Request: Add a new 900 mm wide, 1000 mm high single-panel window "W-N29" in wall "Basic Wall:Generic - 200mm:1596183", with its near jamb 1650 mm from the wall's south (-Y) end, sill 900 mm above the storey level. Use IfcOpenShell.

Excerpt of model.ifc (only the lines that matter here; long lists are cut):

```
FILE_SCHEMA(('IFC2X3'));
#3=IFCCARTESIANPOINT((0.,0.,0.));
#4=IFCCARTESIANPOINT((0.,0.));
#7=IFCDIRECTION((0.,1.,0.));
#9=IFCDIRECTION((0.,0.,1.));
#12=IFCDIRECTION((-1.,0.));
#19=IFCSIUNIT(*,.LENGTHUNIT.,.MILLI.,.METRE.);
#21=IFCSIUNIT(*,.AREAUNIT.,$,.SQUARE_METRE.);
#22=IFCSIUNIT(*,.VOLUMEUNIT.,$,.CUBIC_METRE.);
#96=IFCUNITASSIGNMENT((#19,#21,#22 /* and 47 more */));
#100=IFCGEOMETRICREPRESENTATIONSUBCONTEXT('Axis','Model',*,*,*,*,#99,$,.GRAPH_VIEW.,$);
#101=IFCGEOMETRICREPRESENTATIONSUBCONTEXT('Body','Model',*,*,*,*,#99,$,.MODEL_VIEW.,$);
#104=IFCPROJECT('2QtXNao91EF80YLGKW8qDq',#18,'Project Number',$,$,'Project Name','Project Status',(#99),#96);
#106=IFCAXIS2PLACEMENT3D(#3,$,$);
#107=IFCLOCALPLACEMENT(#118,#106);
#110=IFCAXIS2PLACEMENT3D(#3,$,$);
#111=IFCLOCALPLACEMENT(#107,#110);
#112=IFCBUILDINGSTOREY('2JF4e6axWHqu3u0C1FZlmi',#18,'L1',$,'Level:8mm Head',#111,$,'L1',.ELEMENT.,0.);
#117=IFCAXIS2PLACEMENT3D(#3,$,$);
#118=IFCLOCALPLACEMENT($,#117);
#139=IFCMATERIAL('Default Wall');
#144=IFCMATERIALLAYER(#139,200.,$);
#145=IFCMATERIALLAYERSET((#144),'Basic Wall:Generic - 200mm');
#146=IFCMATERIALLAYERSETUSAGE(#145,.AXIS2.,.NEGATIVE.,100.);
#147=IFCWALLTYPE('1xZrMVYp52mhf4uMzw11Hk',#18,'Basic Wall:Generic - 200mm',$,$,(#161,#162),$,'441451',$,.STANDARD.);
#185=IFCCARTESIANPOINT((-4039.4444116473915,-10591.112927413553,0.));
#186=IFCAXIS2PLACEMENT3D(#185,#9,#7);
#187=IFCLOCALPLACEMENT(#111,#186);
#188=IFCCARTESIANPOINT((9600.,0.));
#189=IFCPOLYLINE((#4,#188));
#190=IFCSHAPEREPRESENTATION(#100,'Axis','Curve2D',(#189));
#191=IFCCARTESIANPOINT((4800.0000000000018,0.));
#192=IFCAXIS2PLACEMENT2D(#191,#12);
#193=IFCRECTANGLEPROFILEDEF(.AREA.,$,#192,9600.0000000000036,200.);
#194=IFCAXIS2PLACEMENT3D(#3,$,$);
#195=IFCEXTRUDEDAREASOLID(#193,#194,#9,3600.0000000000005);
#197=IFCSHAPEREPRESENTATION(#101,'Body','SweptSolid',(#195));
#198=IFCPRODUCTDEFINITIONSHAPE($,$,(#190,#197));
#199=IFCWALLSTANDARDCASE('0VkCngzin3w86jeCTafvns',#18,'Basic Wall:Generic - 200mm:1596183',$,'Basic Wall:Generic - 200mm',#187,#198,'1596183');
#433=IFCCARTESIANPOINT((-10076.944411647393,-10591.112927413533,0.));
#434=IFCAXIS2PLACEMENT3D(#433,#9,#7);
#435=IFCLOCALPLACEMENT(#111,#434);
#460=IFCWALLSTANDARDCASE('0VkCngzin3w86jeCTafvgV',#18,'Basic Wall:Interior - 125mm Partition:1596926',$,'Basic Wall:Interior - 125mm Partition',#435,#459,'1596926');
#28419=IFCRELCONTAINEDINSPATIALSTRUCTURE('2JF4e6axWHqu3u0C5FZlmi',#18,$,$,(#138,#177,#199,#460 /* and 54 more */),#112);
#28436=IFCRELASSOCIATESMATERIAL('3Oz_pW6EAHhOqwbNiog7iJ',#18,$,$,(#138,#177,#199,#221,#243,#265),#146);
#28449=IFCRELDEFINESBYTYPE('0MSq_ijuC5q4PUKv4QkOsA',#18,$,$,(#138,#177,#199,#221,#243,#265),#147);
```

```python
import numpy as np
import ifcopenshell
import ifcopenshell.api.feature
import ifcopenshell.api.geometry
import ifcopenshell.api.root
import ifcopenshell.api.spatial
import ifcopenshell.api.type
import ifcopenshell.geom
import ifcopenshell.util.element
import ifcopenshell.util.placement
import ifcopenshell.util.representation
import ifcopenshell.util.shape
import ifcopenshell.util.unit

model = ifcopenshell.open("model.ifc")
unit_scale = ifcopenshell.util.unit.calculate_unit_scale(model)
settings = ifcopenshell.geom.settings()


def volume(element):
    """Net volume in cubic metres, openings subtracted."""
    shape = ifcopenshell.geom.create_shape(settings, element)
    return ifcopenshell.util.shape.get_volume(shape.geometry)


wall = model.by_guid("0VkCngzin3w86jeCTafvns")
storey = ifcopenshell.util.element.get_container(wall, ifc_class="IfcBuildingStorey")
context = ifcopenshell.util.representation.get_context(model, "Model", "Body", "MODEL_VIEW")
before = volume(wall)

width, height, from_end, sill = 0.9, 1, 1.65, 0.9  # metres

# The wall runs along its own X axis, and the end named is its -X end.
wall_shape = ifcopenshell.geom.create_shape(settings, wall)
x, y, z = ifcopenshell.util.shape.get_vertices(wall_shape.geometry).T
start = x.min() + from_end
face, thickness = float(y.min()), float(y.max() - y.min())
wall_matrix = ifcopenshell.util.placement.get_local_placement(wall.ObjectPlacement)
level = ifcopenshell.util.placement.get_local_placement(storey.ObjectPlacement)[2, 3]


def in_wall(x, y):
    """Placement at x, y metres in the wall's axes, at sill height."""
    matrix = wall_matrix.copy()
    matrix[:, 3] = wall_matrix @ np.array([x / unit_scale, y / unit_scale, 0.0, 1.0])
    matrix[2, 3] = level + sill / unit_scale
    return matrix


# Opening: a box that overshoots both wall faces by 50 mm.
opening = ifcopenshell.api.root.create_entity(model, ifc_class="IfcOpeningElement")
box = ifcopenshell.api.geometry.add_wall_representation(
    model, context=context, length=width, height=height, thickness=thickness + 0.1
)
ifcopenshell.api.geometry.assign_representation(model, product=opening, representation=box)
ifcopenshell.api.geometry.edit_object_placement(model, product=opening, matrix=in_wall(start, face - 0.05), is_si=False)
ifcopenshell.api.feature.add_feature(model, feature=opening, element=wall)

window = ifcopenshell.api.root.create_entity(model, ifc_class="IfcWindow", name="W-N29")
window.OverallWidth, window.OverallHeight = width / unit_scale, height / unit_scale
body = ifcopenshell.api.geometry.add_window_representation(
    model,
    context=context,
    overall_width=window.OverallWidth,
    overall_height=window.OverallHeight,
    partition_type="SINGLE_PANEL",
)
ifcopenshell.api.geometry.assign_representation(model, product=window, representation=body)
ifcopenshell.api.spatial.assign_container(model, products=[window], relating_structure=storey)
fills = ifcopenshell.api.feature.add_filling(model, opening=opening, element=window)
fills.OwnerHistory = window.OwnerHistory  # required in IFC2X3

# IFC2X3 keeps the operation on the window style.
style = ifcopenshell.api.root.create_entity(model, ifc_class="IfcWindowStyle", name="W-N29")
style.OperationType, style.ConstructionType = "SINGLE_PANEL", "NOTDEFINED"
style.ParameterTakesPrecedence = style.Sizeable = False
ifcopenshell.api.type.assign_type(model, related_objects=[window], relating_type=style)

# Centre the window in the wall's thickness.
ifcopenshell.api.geometry.edit_object_placement(model, product=window, matrix=in_wall(start, face), is_si=False)
window_shape = ifcopenshell.geom.create_shape(settings, window)
depth = ifcopenshell.util.shape.get_vertices(window_shape.geometry)[:, 1]
offset = face + thickness / 2 - (depth.min() + depth.max()) / 2
ifcopenshell.api.geometry.edit_object_placement(model, product=window, matrix=in_wall(start, offset), is_si=False)

after = volume(wall)

print(f"wall volume {before:.3f} -> {after:.3f} m3")

model.write("model_v2.ifc")
```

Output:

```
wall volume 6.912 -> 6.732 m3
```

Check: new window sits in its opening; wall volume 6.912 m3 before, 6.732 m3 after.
